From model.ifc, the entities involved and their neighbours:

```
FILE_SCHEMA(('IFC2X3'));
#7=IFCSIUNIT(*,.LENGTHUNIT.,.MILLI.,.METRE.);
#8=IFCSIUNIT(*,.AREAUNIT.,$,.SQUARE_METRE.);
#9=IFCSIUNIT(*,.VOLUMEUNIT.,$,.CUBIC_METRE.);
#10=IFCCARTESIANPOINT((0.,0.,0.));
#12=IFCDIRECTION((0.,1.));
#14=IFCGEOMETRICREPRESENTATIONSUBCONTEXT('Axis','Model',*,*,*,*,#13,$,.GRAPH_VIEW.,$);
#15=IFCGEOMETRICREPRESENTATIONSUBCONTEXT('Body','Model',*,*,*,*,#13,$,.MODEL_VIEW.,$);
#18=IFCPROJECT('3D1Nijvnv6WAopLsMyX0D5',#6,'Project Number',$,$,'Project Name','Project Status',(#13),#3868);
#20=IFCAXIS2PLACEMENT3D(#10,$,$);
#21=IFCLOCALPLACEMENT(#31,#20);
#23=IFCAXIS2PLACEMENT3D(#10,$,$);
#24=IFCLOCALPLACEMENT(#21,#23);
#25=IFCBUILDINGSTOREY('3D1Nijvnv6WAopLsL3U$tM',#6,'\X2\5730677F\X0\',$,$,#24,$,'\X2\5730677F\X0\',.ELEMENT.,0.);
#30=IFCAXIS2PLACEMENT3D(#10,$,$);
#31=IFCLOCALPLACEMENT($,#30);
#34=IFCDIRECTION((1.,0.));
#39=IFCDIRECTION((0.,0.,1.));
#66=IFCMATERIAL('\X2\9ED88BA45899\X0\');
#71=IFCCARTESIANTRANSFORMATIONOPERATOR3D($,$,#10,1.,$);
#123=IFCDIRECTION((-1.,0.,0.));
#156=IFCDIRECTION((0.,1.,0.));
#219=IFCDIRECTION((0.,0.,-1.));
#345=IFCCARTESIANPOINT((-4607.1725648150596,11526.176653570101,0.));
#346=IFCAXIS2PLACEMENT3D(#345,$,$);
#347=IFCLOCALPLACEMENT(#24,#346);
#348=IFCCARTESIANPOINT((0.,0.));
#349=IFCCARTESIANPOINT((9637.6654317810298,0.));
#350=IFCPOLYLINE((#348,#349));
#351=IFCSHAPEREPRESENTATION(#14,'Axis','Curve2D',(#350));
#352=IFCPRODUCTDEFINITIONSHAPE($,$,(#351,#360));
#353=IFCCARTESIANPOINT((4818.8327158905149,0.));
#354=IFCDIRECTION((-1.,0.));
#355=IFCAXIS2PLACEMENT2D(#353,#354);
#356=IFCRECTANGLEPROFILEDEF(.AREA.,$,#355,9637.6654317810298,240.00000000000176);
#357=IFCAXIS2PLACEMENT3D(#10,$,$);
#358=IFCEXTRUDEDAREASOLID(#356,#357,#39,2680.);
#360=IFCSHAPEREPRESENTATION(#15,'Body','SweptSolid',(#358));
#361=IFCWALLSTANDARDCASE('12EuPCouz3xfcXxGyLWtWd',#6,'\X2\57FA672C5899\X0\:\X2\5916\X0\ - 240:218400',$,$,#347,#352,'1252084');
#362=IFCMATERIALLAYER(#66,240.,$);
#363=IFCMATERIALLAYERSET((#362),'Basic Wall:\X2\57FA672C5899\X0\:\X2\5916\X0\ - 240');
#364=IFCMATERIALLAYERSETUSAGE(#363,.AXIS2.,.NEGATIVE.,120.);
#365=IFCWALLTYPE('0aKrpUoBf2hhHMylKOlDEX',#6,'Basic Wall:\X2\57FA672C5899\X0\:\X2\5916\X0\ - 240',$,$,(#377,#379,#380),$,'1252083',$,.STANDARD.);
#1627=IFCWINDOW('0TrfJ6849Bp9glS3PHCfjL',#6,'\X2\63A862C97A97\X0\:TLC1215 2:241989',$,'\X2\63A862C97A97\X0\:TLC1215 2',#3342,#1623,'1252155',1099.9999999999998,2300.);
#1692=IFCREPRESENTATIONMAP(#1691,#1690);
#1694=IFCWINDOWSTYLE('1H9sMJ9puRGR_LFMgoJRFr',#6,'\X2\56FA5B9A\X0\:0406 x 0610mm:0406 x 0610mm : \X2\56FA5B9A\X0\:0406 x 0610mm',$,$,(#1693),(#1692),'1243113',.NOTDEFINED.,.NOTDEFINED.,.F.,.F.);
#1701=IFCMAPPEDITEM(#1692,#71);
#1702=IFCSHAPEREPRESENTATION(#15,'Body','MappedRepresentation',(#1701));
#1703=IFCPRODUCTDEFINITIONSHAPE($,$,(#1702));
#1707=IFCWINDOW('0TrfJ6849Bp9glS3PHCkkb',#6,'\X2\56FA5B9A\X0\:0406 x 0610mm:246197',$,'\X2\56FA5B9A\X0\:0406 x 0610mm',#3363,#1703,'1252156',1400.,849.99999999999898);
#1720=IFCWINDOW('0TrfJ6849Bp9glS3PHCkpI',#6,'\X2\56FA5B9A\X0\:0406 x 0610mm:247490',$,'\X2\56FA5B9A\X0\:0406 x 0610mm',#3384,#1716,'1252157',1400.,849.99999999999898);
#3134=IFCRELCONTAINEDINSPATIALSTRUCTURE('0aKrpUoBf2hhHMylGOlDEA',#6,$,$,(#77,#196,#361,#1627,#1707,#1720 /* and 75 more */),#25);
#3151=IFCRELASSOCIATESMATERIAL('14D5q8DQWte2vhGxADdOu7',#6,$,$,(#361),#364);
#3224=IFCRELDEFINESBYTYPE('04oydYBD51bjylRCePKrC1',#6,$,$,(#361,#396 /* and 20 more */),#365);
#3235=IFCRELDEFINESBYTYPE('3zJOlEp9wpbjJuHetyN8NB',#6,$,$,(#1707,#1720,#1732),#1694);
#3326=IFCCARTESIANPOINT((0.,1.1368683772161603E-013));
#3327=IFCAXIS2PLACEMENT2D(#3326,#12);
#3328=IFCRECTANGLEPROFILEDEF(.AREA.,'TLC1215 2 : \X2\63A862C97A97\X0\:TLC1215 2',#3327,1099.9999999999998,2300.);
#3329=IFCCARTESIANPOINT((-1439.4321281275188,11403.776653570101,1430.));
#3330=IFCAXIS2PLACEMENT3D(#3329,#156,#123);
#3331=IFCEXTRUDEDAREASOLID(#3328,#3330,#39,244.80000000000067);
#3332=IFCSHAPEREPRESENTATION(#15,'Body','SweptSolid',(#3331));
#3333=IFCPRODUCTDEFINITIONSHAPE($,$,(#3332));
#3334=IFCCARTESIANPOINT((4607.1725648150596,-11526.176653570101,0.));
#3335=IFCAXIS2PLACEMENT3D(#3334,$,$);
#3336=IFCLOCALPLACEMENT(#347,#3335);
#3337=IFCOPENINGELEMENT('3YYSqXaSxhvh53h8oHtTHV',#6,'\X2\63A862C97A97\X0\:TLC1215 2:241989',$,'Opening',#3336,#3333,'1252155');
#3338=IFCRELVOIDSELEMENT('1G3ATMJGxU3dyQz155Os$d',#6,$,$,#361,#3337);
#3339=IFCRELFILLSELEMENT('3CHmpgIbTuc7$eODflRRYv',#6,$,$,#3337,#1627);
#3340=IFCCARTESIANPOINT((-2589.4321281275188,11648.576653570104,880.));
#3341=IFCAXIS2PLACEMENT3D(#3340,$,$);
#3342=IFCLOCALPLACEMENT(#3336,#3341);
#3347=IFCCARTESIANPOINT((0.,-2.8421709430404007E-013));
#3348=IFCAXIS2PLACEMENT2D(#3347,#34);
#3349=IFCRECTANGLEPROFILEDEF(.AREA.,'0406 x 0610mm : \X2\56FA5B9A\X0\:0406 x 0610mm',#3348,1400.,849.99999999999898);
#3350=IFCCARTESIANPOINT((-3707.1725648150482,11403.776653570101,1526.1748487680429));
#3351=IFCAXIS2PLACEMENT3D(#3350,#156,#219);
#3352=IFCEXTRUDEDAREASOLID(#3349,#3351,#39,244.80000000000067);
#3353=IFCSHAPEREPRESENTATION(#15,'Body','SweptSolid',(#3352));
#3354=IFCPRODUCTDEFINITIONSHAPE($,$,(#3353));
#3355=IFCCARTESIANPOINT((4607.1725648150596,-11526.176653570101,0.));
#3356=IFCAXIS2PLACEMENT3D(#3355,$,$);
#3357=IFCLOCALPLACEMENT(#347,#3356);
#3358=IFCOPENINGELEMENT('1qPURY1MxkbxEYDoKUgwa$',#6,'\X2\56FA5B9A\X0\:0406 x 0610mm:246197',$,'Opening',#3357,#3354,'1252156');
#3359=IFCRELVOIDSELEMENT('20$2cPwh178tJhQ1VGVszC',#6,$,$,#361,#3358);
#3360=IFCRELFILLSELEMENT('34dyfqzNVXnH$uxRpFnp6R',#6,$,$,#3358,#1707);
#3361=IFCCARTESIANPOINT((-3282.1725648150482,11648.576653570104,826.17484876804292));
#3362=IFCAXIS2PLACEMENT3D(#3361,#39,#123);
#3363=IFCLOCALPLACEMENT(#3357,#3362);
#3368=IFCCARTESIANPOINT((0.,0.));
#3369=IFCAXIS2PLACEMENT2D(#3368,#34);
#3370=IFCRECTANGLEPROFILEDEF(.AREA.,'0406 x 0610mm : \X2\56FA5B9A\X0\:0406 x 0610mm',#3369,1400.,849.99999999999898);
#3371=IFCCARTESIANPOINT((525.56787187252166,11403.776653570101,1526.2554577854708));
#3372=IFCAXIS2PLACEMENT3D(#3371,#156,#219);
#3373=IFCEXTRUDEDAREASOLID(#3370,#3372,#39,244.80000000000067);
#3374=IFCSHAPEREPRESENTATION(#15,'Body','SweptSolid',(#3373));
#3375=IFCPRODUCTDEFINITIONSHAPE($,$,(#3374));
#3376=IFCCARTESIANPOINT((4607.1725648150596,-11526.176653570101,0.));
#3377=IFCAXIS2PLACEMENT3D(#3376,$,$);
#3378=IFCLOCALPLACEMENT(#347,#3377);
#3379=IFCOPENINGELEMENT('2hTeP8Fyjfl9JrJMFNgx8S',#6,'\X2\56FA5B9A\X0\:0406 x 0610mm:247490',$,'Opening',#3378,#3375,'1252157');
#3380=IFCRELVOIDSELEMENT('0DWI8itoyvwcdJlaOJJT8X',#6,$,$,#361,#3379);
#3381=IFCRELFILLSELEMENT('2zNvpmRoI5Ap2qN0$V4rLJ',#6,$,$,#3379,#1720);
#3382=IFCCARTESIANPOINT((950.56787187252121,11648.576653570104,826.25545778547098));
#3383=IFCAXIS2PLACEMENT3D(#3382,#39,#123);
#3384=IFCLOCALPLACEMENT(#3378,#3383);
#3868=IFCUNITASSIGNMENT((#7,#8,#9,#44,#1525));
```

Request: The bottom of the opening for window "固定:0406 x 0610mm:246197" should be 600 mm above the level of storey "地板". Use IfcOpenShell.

```python
import numpy as np
import ifcopenshell
import ifcopenshell.api.geometry
import ifcopenshell.geom
import ifcopenshell.util.element
import ifcopenshell.util.placement
import ifcopenshell.util.shape
import ifcopenshell.util.unit

model = ifcopenshell.open("model.ifc")
unit_scale = ifcopenshell.util.unit.calculate_unit_scale(model)

window = model.by_guid("0TrfJ6849Bp9glS3PHCkkb")
opening = window.FillsVoids[0].RelatingOpeningElement
storey = ifcopenshell.util.element.get_container(window, ifc_class="IfcBuildingStorey")
level = ifcopenshell.util.placement.get_local_placement(storey.ObjectPlacement)[2, 3]

# The opening's origin need not be at the sill, so measure its lowest point.
shape = ifcopenshell.geom.create_shape(ifcopenshell.geom.settings(), opening)
bottom = ifcopenshell.util.shape.get_shape_bottom_elevation(shape, shape.geometry) / unit_scale
dz = level + 0.6 / unit_scale - bottom

shift = np.array([0.0, 0.0, dz])
# The window is placed relative to its opening, so it follows when the opening moves.
matrix = ifcopenshell.util.placement.get_local_placement(opening.ObjectPlacement)
matrix[:3, 3] += shift
ifcopenshell.api.geometry.edit_object_placement(
    model, product=opening, matrix=matrix, is_si=False, should_transform_children=True
)

print(f"moved by {dz * unit_scale:+.3f} m")

model.write("model-out.ifc")
```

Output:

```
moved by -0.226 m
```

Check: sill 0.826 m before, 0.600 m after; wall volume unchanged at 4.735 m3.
